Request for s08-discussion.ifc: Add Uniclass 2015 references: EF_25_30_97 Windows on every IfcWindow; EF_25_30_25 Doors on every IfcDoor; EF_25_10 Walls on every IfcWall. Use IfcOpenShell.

First a look at what the model holds.

```python
import ifcopenshell

model = ifcopenshell.open("s08-discussion.ifc")
print(model.schema)
print("classifications:", [c.Name for c in model.by_type("IfcClassification")])
for ifc_class in ("IfcDoor", "IfcRoof", "IfcStair", "IfcWall", "IfcWindow"):
    print(ifc_class, len(model.by_type(ifc_class)))
```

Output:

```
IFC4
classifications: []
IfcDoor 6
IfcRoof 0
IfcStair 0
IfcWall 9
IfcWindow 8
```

```python
import ifcopenshell
import ifcopenshell.api.classification

model = ifcopenshell.open("s08-discussion.ifc")

system = ifcopenshell.api.classification.add_classification(model, classification="Uniclass 2015")

codes = {
    "IfcWindow": ("EF_25_30_97", "Windows"),
    "IfcDoor": ("EF_25_30_25", "Doors"),
    "IfcWall": ("EF_25_10", "Walls"),
}
for ifc_class, (code, name) in codes.items():
    products = model.by_type(ifc_class)
    ifcopenshell.api.classification.add_reference(
        model, products=products, classification=system, identification=code, name=name
    )
    print(code, len(products))

model.write("s08-discussion_edited.ifc")
```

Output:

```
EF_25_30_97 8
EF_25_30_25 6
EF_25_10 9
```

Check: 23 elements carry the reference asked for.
